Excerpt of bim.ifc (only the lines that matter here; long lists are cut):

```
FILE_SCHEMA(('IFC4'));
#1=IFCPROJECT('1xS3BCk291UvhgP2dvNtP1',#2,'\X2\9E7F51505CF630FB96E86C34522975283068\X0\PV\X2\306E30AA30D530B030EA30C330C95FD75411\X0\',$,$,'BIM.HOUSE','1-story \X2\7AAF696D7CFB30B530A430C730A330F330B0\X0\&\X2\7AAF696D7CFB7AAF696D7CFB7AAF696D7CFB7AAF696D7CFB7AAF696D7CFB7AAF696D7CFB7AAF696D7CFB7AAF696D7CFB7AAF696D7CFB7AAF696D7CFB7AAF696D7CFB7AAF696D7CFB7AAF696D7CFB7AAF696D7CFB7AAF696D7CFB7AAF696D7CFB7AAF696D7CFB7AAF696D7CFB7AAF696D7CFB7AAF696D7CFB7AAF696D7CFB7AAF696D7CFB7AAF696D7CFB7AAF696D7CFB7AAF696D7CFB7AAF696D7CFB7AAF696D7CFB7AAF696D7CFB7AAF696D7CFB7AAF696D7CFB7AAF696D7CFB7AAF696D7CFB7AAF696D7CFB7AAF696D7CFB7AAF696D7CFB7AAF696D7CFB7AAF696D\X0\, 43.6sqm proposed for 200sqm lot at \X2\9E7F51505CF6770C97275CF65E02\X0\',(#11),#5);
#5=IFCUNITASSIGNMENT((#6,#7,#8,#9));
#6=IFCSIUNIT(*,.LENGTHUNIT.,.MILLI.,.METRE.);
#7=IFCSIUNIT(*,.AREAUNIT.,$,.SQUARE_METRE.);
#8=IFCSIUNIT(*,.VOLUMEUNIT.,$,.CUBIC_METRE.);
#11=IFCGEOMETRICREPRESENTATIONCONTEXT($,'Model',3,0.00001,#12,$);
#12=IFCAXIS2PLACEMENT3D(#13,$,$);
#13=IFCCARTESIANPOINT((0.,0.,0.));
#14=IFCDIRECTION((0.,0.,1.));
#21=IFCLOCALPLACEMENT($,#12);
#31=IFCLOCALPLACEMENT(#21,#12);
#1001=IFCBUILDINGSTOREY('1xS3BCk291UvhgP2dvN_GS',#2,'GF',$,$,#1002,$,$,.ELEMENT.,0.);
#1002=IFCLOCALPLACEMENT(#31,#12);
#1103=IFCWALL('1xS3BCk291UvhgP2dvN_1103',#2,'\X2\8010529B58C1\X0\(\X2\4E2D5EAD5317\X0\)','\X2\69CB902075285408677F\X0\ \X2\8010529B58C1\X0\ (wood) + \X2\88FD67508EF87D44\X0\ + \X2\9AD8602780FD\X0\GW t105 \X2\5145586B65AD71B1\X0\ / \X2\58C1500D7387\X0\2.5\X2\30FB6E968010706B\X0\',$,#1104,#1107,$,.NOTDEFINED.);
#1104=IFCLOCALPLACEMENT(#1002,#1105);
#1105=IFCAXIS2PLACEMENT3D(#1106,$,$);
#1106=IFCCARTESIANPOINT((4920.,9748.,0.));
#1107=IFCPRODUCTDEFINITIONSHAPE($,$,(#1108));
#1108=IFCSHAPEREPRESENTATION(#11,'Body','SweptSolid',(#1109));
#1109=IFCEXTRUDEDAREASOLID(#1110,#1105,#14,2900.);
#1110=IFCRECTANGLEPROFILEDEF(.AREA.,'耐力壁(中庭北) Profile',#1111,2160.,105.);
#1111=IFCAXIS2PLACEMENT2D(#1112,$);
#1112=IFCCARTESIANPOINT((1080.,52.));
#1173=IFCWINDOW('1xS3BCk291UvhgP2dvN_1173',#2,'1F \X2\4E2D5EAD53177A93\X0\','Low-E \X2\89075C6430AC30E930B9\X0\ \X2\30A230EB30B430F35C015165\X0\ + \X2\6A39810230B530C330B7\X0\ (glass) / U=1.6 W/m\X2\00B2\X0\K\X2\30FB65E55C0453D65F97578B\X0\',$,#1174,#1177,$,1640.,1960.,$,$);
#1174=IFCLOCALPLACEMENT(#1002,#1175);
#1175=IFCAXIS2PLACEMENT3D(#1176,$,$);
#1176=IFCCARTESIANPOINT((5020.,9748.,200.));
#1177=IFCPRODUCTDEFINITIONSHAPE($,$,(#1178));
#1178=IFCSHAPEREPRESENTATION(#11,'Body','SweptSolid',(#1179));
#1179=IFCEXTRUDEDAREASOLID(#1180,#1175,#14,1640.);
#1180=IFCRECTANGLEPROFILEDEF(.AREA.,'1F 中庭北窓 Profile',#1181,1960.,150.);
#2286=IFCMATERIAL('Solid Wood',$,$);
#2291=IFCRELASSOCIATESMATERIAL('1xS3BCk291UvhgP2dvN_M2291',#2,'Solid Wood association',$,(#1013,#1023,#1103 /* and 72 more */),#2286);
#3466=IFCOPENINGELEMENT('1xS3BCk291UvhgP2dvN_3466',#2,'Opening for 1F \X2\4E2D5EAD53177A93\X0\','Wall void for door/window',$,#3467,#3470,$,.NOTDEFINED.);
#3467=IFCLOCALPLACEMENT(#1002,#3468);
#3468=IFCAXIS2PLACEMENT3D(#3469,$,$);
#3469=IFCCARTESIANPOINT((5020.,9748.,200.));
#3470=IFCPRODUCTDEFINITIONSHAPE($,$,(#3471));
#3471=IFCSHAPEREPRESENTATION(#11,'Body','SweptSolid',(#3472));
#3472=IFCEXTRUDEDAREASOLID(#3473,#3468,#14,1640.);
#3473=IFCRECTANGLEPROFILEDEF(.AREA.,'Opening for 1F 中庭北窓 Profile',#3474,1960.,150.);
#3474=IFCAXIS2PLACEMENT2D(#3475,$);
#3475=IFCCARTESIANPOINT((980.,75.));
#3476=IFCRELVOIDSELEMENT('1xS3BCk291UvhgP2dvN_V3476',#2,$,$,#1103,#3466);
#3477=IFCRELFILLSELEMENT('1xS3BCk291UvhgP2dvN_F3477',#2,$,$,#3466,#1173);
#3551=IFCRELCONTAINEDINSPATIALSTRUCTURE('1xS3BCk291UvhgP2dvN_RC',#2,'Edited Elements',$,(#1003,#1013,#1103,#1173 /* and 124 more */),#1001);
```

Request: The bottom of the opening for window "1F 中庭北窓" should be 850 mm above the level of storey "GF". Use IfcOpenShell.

```python
import numpy as np
import ifcopenshell
import ifcopenshell.api.geometry
import ifcopenshell.geom
import ifcopenshell.util.element
import ifcopenshell.util.placement
import ifcopenshell.util.shape
import ifcopenshell.util.unit

model = ifcopenshell.open("bim.ifc")
unit_scale = ifcopenshell.util.unit.calculate_unit_scale(model)

window = model.by_guid("1xS3BCk291UvhgP2dvN_1173")
opening = window.FillsVoids[0].RelatingOpeningElement
storey = ifcopenshell.util.element.get_container(window, ifc_class="IfcBuildingStorey")
level = ifcopenshell.util.placement.get_local_placement(storey.ObjectPlacement)[2, 3]

# The opening's origin need not be at the sill, so measure its lowest point.
shape = ifcopenshell.geom.create_shape(ifcopenshell.geom.settings(), opening)
bottom = ifcopenshell.util.shape.get_shape_bottom_elevation(shape, shape.geometry) / unit_scale
dz = level + 0.85 / unit_scale - bottom

shift = np.array([0.0, 0.0, dz])
# The window is not placed relative to its opening, so move both.
for product in (opening, window):
    matrix = ifcopenshell.util.placement.get_local_placement(product.ObjectPlacement)
    matrix[:3, 3] += shift
    ifcopenshell.api.geometry.edit_object_placement(model, product=product, matrix=matrix, is_si=False)

print(f"moved by {dz * unit_scale:+.3f} m")

model.write("bim-out.ifc")
```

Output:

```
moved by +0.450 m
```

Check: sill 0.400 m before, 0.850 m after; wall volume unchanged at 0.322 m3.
